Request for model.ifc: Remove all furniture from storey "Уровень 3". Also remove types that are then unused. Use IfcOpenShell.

First a look at what the model holds.

```python
import ifcopenshell
import ifcopenshell.util.element

model = ifcopenshell.open("model.ifc")
print(model.schema)
storey = next(s for s in model.by_type("IfcBuildingStorey") if s.Name == "Уровень 3")
furniture = [e for e in ifcopenshell.util.element.get_decomposition(storey) if e.is_a("IfcFurnishingElement")]
seen = {}
for e in furniture:
    element_type = ifcopenshell.util.element.get_type(e)
    name = element_type.Name if element_type not in (None, e) else None
    seen[name] = seen.get(name, 0) + 1
for name, count in sorted(seen.items(), key=str):
    print(count, "x", name)
```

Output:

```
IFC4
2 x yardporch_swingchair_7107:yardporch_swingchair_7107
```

```python
import ifcopenshell
import ifcopenshell.api.root
import ifcopenshell.util.element

model = ifcopenshell.open("model.ifc")

storey = next(s for s in model.by_type("IfcBuildingStorey") if s.Name == "Уровень 3")
furniture = [e for e in ifcopenshell.util.element.get_decomposition(storey) if e.is_a("IfcFurnishingElement")]
types = {ifcopenshell.util.element.get_type(e) for e in furniture} - {None, *furniture}

for e in furniture:
    ifcopenshell.api.root.remove_product(model, product=e)
print(len(furniture), "removed")

unused = [t for t in types if not ifcopenshell.util.element.get_types(t)]
for t in unused:
    ifcopenshell.api.root.remove_product(model, product=t)
print(len(unused), "unused types removed")

model.write("model_rev.ifc")
```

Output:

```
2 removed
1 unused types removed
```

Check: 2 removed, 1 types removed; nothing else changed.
